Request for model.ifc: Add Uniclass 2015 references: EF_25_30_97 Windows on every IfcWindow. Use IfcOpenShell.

First a look at what the model holds.

```python
import ifcopenshell

model = ifcopenshell.open("model.ifc")
print(model.schema)
print("classifications:", [c.Name for c in model.by_type("IfcClassification")])
for ifc_class in ("IfcDoor", "IfcRoof", "IfcStair", "IfcWall", "IfcWindow"):
    print(ifc_class, len(model.by_type(ifc_class)))
```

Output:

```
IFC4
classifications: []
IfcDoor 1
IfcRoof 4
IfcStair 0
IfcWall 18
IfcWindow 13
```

```python
import ifcopenshell
import ifcopenshell.api.classification

model = ifcopenshell.open("model.ifc")

system = ifcopenshell.api.classification.add_classification(model, classification="Uniclass 2015")

codes = {
    "IfcWindow": ("EF_25_30_97", "Windows"),
}
for ifc_class, (code, name) in codes.items():
    products = model.by_type(ifc_class)
    ifcopenshell.api.classification.add_reference(
        model, products=products, classification=system, identification=code, name=name
    )
    print(code, len(products))

model.write("model_v2.ifc")
```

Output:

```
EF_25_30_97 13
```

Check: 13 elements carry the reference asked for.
